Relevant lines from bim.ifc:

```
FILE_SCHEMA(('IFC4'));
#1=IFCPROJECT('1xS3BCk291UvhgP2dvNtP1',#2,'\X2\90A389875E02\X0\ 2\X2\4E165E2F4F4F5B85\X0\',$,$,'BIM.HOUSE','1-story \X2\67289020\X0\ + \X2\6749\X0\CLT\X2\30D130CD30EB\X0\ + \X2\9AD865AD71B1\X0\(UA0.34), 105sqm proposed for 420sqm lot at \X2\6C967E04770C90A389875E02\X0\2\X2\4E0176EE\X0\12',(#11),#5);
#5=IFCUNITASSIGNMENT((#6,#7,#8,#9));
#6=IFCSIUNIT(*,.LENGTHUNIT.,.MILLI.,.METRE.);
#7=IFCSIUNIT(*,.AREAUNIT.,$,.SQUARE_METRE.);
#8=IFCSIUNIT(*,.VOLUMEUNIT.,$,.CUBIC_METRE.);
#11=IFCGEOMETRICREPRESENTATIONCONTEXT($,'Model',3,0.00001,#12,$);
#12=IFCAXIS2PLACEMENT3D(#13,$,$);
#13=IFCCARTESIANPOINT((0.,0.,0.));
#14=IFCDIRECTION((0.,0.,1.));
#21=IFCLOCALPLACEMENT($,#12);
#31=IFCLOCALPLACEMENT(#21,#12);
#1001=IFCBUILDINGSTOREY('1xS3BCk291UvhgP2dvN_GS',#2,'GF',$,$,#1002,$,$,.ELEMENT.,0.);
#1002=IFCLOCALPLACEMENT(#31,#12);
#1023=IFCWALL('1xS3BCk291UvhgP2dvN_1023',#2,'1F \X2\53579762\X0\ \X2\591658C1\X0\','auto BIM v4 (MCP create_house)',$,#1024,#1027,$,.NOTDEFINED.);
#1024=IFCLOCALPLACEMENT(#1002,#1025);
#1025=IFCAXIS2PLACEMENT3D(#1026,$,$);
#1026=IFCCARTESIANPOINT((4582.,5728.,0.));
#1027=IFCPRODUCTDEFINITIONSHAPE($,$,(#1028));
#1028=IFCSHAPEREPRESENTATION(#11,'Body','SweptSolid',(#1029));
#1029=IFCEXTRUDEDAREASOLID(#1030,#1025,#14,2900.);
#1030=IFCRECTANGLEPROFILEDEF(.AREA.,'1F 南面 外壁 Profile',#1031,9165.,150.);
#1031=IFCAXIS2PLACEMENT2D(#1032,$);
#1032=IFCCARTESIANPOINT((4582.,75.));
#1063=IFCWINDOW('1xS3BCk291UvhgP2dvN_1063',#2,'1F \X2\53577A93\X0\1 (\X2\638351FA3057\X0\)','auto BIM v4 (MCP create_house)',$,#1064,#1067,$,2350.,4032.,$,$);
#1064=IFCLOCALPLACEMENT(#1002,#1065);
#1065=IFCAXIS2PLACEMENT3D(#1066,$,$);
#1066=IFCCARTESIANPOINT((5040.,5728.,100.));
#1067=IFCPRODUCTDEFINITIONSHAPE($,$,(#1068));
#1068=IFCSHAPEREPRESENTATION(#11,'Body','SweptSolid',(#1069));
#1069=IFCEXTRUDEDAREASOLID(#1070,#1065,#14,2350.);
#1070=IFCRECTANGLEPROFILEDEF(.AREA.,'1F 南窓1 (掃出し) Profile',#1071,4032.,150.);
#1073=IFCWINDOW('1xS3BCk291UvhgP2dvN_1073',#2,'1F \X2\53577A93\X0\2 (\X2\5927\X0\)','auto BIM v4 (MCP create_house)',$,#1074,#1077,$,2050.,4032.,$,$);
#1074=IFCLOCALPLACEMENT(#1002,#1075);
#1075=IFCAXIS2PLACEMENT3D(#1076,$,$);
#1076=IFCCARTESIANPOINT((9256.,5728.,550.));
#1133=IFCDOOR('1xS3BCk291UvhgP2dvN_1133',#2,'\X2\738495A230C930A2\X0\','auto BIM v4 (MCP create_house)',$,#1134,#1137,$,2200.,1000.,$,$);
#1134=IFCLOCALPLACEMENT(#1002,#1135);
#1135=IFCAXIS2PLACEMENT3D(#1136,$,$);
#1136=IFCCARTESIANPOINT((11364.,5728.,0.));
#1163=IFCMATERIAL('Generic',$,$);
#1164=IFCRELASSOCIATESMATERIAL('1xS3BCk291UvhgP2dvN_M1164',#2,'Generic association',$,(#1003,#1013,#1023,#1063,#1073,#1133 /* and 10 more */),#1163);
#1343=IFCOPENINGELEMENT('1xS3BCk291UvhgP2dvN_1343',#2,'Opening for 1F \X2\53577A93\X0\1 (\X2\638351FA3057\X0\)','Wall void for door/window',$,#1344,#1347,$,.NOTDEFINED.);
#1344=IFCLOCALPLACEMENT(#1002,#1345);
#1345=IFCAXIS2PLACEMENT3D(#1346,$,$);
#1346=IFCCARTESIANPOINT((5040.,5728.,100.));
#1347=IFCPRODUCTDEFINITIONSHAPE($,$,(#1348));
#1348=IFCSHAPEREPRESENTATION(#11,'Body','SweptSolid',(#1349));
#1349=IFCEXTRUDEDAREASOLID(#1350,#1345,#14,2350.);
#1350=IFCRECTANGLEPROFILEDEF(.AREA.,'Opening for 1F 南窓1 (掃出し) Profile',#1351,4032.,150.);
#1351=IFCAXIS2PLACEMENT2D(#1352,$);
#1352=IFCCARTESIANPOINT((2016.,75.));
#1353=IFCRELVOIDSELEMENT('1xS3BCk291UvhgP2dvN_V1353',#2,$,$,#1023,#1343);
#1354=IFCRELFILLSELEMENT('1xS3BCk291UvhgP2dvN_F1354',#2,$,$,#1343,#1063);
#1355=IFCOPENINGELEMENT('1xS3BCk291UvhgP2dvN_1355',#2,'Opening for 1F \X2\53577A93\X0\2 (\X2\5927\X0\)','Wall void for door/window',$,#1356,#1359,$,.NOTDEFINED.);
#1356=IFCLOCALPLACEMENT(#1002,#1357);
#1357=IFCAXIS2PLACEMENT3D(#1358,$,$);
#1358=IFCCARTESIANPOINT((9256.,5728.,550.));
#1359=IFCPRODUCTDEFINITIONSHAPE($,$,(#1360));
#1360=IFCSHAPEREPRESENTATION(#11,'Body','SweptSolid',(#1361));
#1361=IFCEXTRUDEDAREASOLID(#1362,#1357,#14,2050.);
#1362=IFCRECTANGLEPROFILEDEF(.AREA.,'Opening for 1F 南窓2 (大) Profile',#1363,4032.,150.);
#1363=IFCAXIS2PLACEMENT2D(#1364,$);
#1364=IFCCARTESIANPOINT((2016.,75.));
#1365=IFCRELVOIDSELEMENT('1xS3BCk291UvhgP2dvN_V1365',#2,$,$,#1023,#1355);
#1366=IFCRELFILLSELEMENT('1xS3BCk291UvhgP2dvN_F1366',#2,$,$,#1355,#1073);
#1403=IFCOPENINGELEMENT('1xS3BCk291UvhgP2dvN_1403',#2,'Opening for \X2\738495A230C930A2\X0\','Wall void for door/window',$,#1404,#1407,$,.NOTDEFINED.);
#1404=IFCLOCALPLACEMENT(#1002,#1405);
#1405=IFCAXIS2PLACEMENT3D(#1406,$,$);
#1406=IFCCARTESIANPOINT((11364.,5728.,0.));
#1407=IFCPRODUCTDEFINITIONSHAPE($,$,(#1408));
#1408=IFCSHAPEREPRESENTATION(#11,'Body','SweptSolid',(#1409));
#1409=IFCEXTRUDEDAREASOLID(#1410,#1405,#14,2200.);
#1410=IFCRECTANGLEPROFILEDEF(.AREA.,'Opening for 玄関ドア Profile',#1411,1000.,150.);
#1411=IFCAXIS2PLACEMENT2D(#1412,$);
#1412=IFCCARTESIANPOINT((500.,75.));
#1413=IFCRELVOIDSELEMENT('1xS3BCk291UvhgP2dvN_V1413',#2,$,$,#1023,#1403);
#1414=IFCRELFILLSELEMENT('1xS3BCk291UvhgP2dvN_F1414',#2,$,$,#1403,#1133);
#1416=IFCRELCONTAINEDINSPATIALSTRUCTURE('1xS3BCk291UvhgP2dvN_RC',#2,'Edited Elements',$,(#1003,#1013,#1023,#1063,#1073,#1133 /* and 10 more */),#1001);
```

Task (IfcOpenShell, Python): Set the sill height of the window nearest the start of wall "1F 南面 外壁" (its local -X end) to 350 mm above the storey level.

```python
import numpy as np
import ifcopenshell
import ifcopenshell.api.geometry
import ifcopenshell.geom
import ifcopenshell.util.element
import ifcopenshell.util.placement
import ifcopenshell.util.shape
import ifcopenshell.util.unit

model = ifcopenshell.open("bim.ifc")
unit_scale = ifcopenshell.util.unit.calculate_unit_scale(model)

window = model.by_guid("1xS3BCk291UvhgP2dvN_1063")
opening = window.FillsVoids[0].RelatingOpeningElement
storey = ifcopenshell.util.element.get_container(window, ifc_class="IfcBuildingStorey")
level = ifcopenshell.util.placement.get_local_placement(storey.ObjectPlacement)[2, 3]

# The opening's origin need not be at the sill, so measure its lowest point.
shape = ifcopenshell.geom.create_shape(ifcopenshell.geom.settings(), opening)
bottom = ifcopenshell.util.shape.get_shape_bottom_elevation(shape, shape.geometry) / unit_scale
dz = level + 350.0 - bottom

shift = np.array([0.0, 0.0, dz])
# The window is not placed relative to its opening, so move both.
for product in (opening, window):
    matrix = ifcopenshell.util.placement.get_local_placement(product.ObjectPlacement)
    matrix[:3, 3] += shift
    ifcopenshell.api.geometry.edit_object_placement(model, product=product, matrix=matrix, is_si=False)

print(f"moved by {dz * unit_scale:+.3f} m")

model.write("bim_rev.ifc")
```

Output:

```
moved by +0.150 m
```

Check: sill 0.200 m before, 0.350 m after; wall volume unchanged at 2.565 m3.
